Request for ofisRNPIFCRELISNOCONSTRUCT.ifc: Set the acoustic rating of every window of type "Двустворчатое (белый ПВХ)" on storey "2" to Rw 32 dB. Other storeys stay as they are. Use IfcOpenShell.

First a look at what the model holds.

```python
import ifcopenshell
import ifcopenshell.util.element

model = ifcopenshell.open("ofisRNPIFCRELISNOCONSTRUCT.ifc")
print(model.schema)
storey = next(s for s in model.by_type("IfcBuildingStorey") if s.Name == "2")
windows = [e for e in ifcopenshell.util.element.get_decomposition(storey) if e.is_a("IfcWindow")]
seen = {}
for e in windows:
    element_type = ifcopenshell.util.element.get_type(e)
    key = (element_type.Name if element_type != e and element_type else None, ifcopenshell.util.element.get_pset(e, "Pset_WindowCommon", "AcousticRating"))
    seen[key] = seen.get(key, 0) + 1
for (name, value), count in sorted(seen.items(), key=str):
    print(count, "x", name, "|", value)
```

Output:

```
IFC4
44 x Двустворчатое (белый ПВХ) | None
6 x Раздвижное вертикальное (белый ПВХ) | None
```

```python
import ifcopenshell
import ifcopenshell.api.pset
import ifcopenshell.util.element

model = ifcopenshell.open("ofisRNPIFCRELISNOCONSTRUCT.ifc")

storey = next(s for s in model.by_type("IfcBuildingStorey") if s.Name == "2")
windows = [e for e in ifcopenshell.util.element.get_decomposition(storey) if e.is_a("IfcWindow")]

count = 0
for e in windows:
    element_type = ifcopenshell.util.element.get_type(e)
    if element_type in (None, e) or element_type.Name != "Двустворчатое (белый ПВХ)":
        continue
    # add_pset returns the element's existing set when there is one.
    pset = ifcopenshell.api.pset.add_pset(model, product=e, name="Pset_WindowCommon")
    ifcopenshell.api.pset.edit_pset(model, pset=pset, properties={"AcousticRating": "Rw 32 dB"})
    count += 1

print(count, "windows updated")

model.write("ofisRNPIFCRELISNOCONSTRUCT_updated.ifc")
```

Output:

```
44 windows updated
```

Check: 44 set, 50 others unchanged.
